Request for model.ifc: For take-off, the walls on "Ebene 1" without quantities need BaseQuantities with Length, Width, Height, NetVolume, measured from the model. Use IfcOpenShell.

First a look at what the model holds.

```python
import ifcopenshell
import ifcopenshell.util.element
import ifcopenshell.util.unit

model = ifcopenshell.open("model.ifc")
print(model.schema)
for unit_type in ("LENGTHUNIT", "AREAUNIT", "VOLUMEUNIT"):
    print(unit_type, ifcopenshell.util.unit.calculate_unit_scale(model, unit_type))
storey = next(s for s in model.by_type("IfcBuildingStorey") if s.Name == "Ebene 1")
walls = [e for e in ifcopenshell.util.element.get_decomposition(storey) if e.is_a("IfcWall")]
for e in sorted(walls, key=lambda e: e.id()):
    print(e.id(), e.is_a(), e.Name, list(ifcopenshell.util.element.get_psets(e, qtos_only=True)), sep=" | ")
```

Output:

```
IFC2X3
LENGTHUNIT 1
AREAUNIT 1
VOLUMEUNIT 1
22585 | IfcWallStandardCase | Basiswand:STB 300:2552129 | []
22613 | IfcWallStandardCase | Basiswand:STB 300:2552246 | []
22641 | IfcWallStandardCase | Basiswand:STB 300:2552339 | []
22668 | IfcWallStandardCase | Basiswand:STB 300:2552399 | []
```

```python
import ifcopenshell
import ifcopenshell.api.pset
import ifcopenshell.geom
import ifcopenshell.util.element
import ifcopenshell.util.shape
import ifcopenshell.util.unit

model = ifcopenshell.open("model.ifc")
unit_scale = ifcopenshell.util.unit.calculate_unit_scale(model)
volume_scale = ifcopenshell.util.unit.calculate_unit_scale(model, "VOLUMEUNIT")
settings = ifcopenshell.geom.settings()

storey = next(s for s in model.by_type("IfcBuildingStorey") if s.Name == "Ebene 1")
walls = [e for e in ifcopenshell.util.element.get_decomposition(storey) if e.is_a("IfcWall")]

for e in sorted(walls, key=lambda e: e.id()):
    if ifcopenshell.util.element.get_psets(e, qtos_only=True, should_inherit=False):
        continue
    # Geometry comes back in metres, in the element's own axes.
    shape = ifcopenshell.geom.create_shape(settings, e)
    values = {
        "Length": ifcopenshell.util.shape.get_x(shape.geometry) / unit_scale,
        "Width": ifcopenshell.util.shape.get_y(shape.geometry) / unit_scale,
        "Height": ifcopenshell.util.shape.get_z(shape.geometry) / unit_scale,
        "NetVolume": ifcopenshell.util.shape.get_volume(shape.geometry) / volume_scale,
    }
    qto = ifcopenshell.api.pset.add_qto(model, product=e, name="BaseQuantities")
    ifcopenshell.api.pset.edit_qto(model, qto=qto, properties=values)
    print(e.id(), {k: round(v, 3) for k, v in values.items()})

model.write("model_v2.ifc")
```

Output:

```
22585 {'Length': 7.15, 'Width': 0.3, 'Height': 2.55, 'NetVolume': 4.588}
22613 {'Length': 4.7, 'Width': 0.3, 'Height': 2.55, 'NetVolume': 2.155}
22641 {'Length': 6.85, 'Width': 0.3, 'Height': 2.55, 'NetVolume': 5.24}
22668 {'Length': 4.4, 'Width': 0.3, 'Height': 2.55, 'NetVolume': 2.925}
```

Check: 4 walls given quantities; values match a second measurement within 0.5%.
